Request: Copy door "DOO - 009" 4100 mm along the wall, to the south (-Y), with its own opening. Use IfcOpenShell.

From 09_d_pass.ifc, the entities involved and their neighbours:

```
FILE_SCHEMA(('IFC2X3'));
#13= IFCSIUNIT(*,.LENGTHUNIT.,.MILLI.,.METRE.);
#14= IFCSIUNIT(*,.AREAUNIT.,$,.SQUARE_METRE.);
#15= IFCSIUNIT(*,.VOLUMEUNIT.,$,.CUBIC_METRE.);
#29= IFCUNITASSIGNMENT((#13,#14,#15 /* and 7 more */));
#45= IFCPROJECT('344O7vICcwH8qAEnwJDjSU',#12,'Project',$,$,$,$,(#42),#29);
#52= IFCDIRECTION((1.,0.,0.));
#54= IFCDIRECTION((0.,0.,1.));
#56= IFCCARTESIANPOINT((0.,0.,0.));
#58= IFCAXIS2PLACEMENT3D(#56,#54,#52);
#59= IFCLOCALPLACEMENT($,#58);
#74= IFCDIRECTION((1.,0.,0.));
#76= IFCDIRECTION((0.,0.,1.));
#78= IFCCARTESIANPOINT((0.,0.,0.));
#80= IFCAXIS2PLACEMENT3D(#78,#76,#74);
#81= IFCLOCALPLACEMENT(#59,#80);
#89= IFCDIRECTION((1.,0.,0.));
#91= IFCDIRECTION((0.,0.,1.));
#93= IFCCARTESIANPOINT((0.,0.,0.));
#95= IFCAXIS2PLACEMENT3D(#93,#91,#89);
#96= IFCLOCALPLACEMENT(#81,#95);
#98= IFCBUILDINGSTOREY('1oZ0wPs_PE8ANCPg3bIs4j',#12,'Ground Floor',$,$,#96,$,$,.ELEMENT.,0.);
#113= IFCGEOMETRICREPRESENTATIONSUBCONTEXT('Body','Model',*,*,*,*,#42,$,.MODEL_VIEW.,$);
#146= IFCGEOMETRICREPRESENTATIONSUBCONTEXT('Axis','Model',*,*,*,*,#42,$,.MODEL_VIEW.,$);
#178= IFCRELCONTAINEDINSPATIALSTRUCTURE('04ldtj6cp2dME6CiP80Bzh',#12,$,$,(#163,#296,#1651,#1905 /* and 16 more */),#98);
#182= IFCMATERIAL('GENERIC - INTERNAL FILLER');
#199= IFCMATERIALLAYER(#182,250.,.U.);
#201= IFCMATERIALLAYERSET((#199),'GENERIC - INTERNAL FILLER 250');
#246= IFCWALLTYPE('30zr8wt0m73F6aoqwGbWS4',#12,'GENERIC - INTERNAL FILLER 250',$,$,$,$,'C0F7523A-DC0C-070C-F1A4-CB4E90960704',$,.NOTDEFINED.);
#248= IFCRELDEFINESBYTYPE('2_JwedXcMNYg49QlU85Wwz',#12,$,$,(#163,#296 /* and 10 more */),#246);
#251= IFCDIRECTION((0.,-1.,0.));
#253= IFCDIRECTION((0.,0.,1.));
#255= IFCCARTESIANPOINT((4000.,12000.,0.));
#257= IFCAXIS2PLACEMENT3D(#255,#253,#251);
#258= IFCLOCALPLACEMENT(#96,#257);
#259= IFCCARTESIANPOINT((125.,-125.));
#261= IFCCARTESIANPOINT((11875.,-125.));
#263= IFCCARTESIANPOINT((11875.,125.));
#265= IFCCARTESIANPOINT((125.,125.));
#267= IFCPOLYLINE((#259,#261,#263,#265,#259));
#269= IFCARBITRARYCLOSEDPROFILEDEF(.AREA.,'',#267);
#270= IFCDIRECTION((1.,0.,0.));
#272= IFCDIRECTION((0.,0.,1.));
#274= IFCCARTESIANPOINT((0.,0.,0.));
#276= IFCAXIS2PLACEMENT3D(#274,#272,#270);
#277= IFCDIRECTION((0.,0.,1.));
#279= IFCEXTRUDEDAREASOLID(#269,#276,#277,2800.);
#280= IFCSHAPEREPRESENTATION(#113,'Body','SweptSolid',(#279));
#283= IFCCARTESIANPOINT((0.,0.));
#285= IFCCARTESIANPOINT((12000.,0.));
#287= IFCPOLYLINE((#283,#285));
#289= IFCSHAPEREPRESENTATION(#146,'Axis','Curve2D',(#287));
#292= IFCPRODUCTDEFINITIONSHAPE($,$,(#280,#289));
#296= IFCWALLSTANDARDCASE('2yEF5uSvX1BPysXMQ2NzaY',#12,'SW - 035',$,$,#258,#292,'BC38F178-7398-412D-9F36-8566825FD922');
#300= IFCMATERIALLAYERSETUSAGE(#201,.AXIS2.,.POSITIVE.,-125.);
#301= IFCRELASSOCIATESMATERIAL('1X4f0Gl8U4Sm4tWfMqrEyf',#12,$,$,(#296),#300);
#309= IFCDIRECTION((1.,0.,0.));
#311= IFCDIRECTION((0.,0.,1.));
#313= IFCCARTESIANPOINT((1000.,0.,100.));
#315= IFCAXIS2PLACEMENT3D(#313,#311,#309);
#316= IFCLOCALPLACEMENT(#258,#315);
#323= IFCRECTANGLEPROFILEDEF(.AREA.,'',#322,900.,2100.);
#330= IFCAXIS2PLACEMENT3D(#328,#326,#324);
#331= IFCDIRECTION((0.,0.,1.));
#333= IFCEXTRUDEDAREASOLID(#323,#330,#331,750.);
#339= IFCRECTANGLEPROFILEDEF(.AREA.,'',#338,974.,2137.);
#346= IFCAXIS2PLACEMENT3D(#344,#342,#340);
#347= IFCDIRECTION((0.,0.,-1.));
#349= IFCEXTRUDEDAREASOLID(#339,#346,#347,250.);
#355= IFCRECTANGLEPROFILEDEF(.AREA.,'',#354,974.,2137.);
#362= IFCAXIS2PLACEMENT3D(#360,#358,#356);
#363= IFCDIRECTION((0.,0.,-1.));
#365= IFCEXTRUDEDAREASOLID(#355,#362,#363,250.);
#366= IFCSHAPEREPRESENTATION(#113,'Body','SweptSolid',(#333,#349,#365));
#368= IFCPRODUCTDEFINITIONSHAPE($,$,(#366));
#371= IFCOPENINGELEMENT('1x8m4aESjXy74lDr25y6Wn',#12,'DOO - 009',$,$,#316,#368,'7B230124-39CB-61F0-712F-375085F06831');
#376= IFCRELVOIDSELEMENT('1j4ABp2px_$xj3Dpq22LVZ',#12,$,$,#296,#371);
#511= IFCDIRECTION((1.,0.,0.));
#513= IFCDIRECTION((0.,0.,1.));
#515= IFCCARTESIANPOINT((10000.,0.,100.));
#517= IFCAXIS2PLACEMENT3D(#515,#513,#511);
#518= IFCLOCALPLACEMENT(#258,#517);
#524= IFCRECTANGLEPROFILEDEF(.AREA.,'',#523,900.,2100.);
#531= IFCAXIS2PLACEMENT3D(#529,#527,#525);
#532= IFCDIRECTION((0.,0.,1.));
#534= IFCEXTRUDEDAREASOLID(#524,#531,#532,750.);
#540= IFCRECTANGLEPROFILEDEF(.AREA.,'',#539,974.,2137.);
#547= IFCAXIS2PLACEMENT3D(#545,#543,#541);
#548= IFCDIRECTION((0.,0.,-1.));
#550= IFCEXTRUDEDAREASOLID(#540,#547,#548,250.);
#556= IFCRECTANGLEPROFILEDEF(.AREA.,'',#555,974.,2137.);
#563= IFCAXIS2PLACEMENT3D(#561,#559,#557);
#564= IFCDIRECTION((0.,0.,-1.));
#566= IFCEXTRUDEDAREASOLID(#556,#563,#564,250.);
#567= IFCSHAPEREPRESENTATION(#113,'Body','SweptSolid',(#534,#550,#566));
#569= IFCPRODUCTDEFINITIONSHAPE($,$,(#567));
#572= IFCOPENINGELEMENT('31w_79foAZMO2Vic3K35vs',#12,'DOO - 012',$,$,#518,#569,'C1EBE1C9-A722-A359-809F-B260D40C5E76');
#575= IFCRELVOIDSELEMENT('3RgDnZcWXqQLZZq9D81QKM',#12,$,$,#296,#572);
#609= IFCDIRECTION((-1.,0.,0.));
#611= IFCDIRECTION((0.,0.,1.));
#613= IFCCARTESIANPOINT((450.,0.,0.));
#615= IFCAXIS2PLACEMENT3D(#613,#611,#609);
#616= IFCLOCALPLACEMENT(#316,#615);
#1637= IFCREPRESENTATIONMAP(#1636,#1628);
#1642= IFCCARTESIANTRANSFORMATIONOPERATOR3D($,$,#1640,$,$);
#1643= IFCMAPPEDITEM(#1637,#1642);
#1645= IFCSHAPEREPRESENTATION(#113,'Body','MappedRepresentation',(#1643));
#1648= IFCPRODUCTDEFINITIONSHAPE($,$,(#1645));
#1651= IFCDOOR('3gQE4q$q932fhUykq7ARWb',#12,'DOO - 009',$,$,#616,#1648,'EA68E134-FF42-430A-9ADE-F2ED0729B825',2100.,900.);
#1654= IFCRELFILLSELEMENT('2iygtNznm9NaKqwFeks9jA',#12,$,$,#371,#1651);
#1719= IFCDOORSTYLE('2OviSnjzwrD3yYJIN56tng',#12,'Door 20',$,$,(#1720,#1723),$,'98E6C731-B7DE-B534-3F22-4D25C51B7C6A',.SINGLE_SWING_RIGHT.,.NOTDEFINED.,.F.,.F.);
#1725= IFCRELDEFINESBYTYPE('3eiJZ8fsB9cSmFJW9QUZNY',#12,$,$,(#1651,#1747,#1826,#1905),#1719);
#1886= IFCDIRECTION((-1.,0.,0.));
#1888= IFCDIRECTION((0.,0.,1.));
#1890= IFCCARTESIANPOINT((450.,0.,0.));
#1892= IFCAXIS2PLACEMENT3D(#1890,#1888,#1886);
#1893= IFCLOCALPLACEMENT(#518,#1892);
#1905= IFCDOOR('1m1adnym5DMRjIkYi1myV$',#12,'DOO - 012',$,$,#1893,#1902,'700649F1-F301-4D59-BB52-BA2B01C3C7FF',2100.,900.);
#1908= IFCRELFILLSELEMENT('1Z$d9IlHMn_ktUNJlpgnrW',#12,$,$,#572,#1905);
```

```python
import ifcopenshell
import ifcopenshell.api.feature
import ifcopenshell.api.geometry
import ifcopenshell.api.root
import ifcopenshell.geom
import ifcopenshell.util.element
import ifcopenshell.util.placement
import ifcopenshell.util.shape
import ifcopenshell.util.unit

model = ifcopenshell.open("09_d_pass.ifc")
unit_scale = ifcopenshell.util.unit.calculate_unit_scale(model)
settings = ifcopenshell.geom.settings()


def volume(element):
    """Net volume in cubic metres, openings subtracted."""
    shape = ifcopenshell.geom.create_shape(settings, element)
    return ifcopenshell.util.shape.get_volume(shape.geometry)


def reuse_history(source, copy):
    """copy_class also copies each property set's owner history, people and application; keep the originals."""
    for rel in copy.IsDefinedBy:
        if rel.is_a("IfcRelDefinesByProperties") and (history := rel.RelatingPropertyDefinition.OwnerHistory):
            rel.RelatingPropertyDefinition.OwnerHistory = source.OwnerHistory
            ifcopenshell.util.element.remove_deep2(model, history)


door = model.by_id(1651)
opening = door.FillsVoids[0].RelatingOpeningElement
wall = opening.VoidsElements[0].RelatingBuildingElement
before = volume(wall)
shift = ifcopenshell.util.placement.get_local_placement(wall.ObjectPlacement)[:3, 0] * 4.1 / unit_scale

# copy_class copies the void relationship, type, container and properties, but no geometry.
new_opening = ifcopenshell.api.root.copy_class(model, product=opening)
new_opening.Representation = ifcopenshell.util.element.copy_deep(
    model, opening.Representation, exclude=["IfcGeometricRepresentationContext", "IfcRepresentationMap"]
)
new_opening.Tag = None
new_door = ifcopenshell.api.root.copy_class(model, product=door)
new_door.Representation = ifcopenshell.util.element.copy_deep(
    model, door.Representation, exclude=["IfcGeometricRepresentationContext", "IfcRepresentationMap"]
)
new_door.Tag = None
reuse_history(door, new_door)
fills = ifcopenshell.api.feature.add_filling(model, opening=new_opening, element=new_door)
fills.OwnerHistory = new_door.OwnerHistory  # required in IFC2X3

for old, new in ((opening, new_opening), (door, new_door)):
    matrix = ifcopenshell.util.placement.get_local_placement(old.ObjectPlacement)
    matrix[:3, 3] += shift
    ifcopenshell.api.geometry.edit_object_placement(model, product=new, matrix=matrix, is_si=False)

after = volume(wall)

print(f"wall volume {before:.3f} -> {after:.3f} m3")

model.write("09_d_pass_edited.ifc")
```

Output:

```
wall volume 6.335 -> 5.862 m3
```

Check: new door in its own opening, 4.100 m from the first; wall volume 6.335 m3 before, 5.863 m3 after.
